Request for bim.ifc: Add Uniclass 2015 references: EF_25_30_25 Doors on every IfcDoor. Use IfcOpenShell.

First a look at what the model holds.

```python
import ifcopenshell

model = ifcopenshell.open("bim.ifc")
print(model.schema)
print("classifications:", [c.Name for c in model.by_type("IfcClassification")])
for ifc_class in ("IfcDoor", "IfcRoof", "IfcStair", "IfcWall", "IfcWindow"):
    print(ifc_class, len(model.by_type(ifc_class)))
```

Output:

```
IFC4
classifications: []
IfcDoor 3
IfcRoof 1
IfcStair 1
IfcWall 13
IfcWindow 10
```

```python
import ifcopenshell
import ifcopenshell.api.classification

model = ifcopenshell.open("bim.ifc")

system = ifcopenshell.api.classification.add_classification(model, classification="Uniclass 2015")

codes = {
    "IfcDoor": ("EF_25_30_25", "Doors"),
}
for ifc_class, (code, name) in codes.items():
    products = model.by_type(ifc_class)
    ifcopenshell.api.classification.add_reference(
        model, products=products, classification=system, identification=code, name=name
    )
    print(code, len(products))

model.write("bim-out.ifc")
```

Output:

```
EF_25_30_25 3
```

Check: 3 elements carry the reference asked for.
